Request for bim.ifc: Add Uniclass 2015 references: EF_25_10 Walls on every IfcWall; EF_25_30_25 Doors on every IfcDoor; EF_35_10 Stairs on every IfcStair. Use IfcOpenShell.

First a look at what the model holds.

```python
import ifcopenshell

model = ifcopenshell.open("bim.ifc")
print(model.schema)
print("classifications:", [c.Name for c in model.by_type("IfcClassification")])
for ifc_class in ("IfcDoor", "IfcRoof", "IfcStair", "IfcWall", "IfcWindow"):
    print(ifc_class, len(model.by_type(ifc_class)))
```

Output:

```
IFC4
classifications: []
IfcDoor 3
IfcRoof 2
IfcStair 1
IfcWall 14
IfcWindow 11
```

```python
import ifcopenshell
import ifcopenshell.api.classification

model = ifcopenshell.open("bim.ifc")

system = ifcopenshell.api.classification.add_classification(model, classification="Uniclass 2015")

codes = {
    "IfcWall": ("EF_25_10", "Walls"),
    "IfcDoor": ("EF_25_30_25", "Doors"),
    "IfcStair": ("EF_35_10", "Stairs"),
}
for ifc_class, (code, name) in codes.items():
    products = model.by_type(ifc_class)
    ifcopenshell.api.classification.add_reference(
        model, products=products, classification=system, identification=code, name=name
    )
    print(code, len(products))

model.write("bim-out.ifc")
```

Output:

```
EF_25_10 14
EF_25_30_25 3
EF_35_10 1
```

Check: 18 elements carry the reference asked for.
